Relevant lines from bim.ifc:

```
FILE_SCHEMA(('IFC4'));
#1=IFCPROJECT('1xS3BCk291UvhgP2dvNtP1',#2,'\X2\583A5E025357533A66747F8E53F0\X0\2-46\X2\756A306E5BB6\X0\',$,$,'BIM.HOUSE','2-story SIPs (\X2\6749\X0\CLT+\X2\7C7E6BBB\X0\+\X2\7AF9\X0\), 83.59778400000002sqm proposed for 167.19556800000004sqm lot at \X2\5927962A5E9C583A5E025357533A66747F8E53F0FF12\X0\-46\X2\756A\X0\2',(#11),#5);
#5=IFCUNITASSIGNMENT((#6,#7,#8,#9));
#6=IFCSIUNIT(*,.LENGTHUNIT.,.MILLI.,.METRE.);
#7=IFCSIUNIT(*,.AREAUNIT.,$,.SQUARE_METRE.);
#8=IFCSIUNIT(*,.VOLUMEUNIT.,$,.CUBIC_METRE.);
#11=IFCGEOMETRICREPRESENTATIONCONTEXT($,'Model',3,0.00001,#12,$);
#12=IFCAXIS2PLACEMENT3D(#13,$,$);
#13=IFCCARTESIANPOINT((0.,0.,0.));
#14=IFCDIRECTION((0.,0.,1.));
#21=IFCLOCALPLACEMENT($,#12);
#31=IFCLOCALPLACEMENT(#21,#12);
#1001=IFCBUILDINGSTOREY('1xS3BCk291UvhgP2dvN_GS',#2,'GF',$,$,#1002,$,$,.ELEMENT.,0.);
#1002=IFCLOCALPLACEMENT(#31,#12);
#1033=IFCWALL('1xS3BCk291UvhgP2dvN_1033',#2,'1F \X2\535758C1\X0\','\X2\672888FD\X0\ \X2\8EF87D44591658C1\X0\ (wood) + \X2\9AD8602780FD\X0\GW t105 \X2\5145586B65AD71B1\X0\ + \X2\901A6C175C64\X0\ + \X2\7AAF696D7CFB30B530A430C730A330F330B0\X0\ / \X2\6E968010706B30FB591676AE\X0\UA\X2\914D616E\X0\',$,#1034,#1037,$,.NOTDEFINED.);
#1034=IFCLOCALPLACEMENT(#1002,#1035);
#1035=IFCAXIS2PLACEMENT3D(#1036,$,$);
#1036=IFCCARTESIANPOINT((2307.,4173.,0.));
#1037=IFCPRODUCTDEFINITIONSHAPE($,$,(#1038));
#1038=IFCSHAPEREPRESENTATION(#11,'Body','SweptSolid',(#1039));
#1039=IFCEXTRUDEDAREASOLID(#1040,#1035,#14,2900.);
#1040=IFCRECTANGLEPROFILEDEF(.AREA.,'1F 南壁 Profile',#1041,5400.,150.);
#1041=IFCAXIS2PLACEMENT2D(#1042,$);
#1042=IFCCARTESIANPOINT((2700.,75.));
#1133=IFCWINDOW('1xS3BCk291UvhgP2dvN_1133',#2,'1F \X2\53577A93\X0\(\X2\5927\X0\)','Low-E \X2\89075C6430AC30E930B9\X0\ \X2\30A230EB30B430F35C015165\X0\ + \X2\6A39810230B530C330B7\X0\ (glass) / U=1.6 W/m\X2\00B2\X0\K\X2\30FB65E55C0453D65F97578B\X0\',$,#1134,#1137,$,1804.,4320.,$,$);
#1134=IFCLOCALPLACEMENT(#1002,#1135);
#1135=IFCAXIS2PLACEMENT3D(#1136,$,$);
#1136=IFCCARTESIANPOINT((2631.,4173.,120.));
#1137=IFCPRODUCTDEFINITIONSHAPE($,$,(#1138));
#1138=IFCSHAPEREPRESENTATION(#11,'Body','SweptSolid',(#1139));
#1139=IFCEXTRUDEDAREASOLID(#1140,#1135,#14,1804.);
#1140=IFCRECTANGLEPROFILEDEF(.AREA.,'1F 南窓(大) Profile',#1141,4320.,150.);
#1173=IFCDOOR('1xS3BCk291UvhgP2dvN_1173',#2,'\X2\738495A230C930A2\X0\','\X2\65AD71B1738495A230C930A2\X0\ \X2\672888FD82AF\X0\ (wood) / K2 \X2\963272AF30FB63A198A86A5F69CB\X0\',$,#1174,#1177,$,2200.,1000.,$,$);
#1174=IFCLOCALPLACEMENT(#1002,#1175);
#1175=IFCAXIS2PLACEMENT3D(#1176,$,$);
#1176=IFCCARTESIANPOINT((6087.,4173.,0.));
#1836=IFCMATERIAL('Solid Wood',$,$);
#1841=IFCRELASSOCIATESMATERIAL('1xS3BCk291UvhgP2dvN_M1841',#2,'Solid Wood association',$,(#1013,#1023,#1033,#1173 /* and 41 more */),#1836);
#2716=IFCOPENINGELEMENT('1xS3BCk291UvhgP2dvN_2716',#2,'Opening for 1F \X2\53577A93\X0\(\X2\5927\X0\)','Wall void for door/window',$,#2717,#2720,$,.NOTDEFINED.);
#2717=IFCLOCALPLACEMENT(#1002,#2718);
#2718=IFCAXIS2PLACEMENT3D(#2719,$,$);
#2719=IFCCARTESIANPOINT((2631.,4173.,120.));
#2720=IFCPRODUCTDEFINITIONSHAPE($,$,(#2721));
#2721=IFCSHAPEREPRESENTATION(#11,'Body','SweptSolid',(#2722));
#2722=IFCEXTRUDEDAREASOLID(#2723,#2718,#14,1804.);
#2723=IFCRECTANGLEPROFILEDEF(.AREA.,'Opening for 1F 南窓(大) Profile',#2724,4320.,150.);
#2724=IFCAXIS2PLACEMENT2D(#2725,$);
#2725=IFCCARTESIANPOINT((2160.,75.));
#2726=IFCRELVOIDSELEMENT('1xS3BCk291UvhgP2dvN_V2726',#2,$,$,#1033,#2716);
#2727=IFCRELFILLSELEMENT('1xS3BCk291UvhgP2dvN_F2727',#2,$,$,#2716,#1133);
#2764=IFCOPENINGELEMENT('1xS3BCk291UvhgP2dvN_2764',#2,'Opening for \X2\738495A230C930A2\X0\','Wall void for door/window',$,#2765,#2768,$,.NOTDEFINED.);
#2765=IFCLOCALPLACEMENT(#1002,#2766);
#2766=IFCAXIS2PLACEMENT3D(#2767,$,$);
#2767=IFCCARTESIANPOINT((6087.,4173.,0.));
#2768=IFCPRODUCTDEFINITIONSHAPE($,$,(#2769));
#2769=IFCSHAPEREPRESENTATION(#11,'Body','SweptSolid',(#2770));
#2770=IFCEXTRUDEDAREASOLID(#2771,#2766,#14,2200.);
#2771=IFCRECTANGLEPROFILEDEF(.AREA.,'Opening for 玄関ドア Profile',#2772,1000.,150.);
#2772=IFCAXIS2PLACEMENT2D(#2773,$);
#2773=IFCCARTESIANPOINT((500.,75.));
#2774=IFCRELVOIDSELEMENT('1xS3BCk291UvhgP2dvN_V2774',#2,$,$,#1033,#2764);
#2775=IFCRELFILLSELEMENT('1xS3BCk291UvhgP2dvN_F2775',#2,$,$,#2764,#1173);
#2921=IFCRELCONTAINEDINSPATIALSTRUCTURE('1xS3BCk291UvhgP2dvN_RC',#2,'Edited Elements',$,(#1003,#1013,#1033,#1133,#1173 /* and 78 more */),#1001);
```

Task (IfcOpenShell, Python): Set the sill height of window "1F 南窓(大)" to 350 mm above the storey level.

```python
import numpy as np
import ifcopenshell
import ifcopenshell.api.geometry
import ifcopenshell.geom
import ifcopenshell.util.element
import ifcopenshell.util.placement
import ifcopenshell.util.shape
import ifcopenshell.util.unit

model = ifcopenshell.open("bim.ifc")
unit_scale = ifcopenshell.util.unit.calculate_unit_scale(model)

window = model.by_guid("1xS3BCk291UvhgP2dvN_1133")
opening = window.FillsVoids[0].RelatingOpeningElement
storey = ifcopenshell.util.element.get_container(window, ifc_class="IfcBuildingStorey")
level = ifcopenshell.util.placement.get_local_placement(storey.ObjectPlacement)[2, 3]

# The opening's origin need not be at the sill, so measure its lowest point.
shape = ifcopenshell.geom.create_shape(ifcopenshell.geom.settings(), opening)
bottom = ifcopenshell.util.shape.get_shape_bottom_elevation(shape, shape.geometry) / unit_scale
dz = level + 350.0 - bottom

shift = np.array([0.0, 0.0, dz])
# The window is not placed relative to its opening, so move both.
for product in (opening, window):
    matrix = ifcopenshell.util.placement.get_local_placement(product.ObjectPlacement)
    matrix[:3, 3] += shift
    ifcopenshell.api.geometry.edit_object_placement(model, product=product, matrix=matrix, is_si=False)

print(f"moved by {dz * unit_scale:+.3f} m")

model.write("bim_edited.ifc")
```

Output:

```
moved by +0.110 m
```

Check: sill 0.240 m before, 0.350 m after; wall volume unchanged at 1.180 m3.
